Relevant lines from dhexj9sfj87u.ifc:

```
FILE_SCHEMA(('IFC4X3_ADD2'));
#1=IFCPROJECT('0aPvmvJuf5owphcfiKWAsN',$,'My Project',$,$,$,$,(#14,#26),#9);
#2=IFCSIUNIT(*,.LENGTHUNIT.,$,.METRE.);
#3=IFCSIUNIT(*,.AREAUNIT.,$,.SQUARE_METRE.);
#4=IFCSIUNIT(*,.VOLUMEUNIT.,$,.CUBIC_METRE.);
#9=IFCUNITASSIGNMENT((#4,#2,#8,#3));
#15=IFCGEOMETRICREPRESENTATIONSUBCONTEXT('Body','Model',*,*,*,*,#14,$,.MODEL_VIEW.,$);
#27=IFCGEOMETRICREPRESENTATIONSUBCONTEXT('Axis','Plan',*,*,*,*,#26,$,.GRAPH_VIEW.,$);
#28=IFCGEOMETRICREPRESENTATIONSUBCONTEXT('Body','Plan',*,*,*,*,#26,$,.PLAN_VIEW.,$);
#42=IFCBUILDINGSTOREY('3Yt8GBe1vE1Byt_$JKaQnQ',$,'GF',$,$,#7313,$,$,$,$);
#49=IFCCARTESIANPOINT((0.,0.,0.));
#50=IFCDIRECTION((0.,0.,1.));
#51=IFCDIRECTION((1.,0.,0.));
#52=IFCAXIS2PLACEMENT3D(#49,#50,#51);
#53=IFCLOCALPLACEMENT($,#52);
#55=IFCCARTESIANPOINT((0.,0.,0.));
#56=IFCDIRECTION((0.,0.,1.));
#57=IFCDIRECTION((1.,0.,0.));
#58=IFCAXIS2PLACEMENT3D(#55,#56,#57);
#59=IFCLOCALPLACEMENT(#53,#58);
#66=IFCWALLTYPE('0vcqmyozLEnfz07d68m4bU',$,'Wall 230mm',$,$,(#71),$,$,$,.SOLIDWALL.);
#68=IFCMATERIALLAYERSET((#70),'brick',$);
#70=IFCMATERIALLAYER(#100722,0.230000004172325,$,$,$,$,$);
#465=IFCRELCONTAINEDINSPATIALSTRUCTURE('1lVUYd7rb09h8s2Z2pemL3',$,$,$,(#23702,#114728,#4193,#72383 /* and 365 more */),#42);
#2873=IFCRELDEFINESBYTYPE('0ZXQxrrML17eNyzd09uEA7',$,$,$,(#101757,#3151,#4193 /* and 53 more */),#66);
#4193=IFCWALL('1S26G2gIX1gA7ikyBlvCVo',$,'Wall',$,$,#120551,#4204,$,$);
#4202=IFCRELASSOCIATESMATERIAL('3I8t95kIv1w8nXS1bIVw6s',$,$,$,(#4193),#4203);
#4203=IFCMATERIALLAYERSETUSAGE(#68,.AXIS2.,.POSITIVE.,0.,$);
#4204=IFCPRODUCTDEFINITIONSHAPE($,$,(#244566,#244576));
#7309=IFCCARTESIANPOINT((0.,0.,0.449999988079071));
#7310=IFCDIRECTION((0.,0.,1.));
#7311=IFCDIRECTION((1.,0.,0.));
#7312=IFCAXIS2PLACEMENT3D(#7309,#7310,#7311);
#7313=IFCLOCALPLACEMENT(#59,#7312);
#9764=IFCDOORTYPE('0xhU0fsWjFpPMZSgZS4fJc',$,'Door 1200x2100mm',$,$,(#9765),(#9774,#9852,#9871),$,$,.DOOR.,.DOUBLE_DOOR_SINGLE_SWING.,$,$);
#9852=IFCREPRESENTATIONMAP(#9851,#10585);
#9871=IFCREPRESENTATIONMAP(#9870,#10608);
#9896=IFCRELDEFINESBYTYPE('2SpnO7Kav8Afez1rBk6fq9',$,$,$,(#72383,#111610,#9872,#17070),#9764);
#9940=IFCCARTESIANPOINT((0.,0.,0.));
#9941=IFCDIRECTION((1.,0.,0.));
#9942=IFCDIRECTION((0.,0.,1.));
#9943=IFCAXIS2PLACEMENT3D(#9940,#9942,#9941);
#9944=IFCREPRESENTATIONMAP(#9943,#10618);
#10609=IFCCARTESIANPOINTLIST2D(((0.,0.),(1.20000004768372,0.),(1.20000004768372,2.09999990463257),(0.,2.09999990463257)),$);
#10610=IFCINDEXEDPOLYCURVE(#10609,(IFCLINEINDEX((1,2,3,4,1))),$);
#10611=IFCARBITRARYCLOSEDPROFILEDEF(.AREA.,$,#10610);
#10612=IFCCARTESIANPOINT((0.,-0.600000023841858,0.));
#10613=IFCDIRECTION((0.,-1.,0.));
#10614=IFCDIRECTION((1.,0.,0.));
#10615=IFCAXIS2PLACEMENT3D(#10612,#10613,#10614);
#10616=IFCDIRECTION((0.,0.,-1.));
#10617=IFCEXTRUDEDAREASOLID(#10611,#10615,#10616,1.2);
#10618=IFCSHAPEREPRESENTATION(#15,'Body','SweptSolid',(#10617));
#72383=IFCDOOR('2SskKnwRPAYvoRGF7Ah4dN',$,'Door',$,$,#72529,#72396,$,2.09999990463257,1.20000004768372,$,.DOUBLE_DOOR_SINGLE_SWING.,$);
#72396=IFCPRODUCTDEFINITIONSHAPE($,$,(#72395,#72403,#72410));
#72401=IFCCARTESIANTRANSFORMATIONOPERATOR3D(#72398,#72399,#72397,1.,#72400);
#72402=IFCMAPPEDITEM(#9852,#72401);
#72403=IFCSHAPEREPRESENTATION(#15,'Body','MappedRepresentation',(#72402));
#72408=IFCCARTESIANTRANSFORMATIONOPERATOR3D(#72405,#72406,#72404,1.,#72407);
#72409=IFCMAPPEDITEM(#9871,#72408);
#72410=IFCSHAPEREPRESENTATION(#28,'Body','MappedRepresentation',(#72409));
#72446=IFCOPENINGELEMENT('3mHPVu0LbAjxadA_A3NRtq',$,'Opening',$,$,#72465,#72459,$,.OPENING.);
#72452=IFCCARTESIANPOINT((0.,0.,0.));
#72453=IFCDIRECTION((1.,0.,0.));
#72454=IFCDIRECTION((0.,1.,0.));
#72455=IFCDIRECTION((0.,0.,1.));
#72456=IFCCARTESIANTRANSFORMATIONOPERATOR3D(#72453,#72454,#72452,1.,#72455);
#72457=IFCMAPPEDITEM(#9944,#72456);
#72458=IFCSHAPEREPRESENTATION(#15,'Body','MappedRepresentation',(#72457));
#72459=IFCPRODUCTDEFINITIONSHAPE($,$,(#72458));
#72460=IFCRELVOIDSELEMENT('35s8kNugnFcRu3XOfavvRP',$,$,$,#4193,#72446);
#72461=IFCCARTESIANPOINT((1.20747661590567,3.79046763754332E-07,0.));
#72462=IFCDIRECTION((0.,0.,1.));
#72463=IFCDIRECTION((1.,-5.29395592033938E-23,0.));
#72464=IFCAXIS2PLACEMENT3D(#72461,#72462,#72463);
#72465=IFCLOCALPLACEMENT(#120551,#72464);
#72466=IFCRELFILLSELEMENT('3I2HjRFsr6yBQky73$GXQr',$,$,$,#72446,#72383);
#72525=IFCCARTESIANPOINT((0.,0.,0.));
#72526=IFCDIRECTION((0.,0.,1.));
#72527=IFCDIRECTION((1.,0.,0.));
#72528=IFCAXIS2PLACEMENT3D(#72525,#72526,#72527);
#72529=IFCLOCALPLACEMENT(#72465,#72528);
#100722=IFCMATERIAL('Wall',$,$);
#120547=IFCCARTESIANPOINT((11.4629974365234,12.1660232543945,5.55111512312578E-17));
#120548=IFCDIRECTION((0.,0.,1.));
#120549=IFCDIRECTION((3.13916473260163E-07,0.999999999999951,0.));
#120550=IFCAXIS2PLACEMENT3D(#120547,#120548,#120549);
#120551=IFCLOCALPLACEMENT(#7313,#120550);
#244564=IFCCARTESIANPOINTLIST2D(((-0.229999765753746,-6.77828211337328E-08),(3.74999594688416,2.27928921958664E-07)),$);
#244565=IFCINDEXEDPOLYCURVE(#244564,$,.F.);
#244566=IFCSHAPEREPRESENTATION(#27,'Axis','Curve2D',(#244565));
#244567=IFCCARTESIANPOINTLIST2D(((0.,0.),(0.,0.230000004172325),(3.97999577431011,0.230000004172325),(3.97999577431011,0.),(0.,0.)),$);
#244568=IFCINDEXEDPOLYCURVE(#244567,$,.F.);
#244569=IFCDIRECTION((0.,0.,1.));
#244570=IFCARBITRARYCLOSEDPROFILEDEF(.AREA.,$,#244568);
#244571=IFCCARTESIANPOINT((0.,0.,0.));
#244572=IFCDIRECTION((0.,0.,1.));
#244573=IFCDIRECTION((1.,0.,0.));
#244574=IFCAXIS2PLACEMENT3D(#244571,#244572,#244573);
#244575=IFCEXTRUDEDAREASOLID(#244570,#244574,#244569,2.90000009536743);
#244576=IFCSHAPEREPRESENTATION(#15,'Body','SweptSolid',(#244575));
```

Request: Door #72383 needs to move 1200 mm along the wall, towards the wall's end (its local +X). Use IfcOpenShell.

```python
import ifcopenshell
import ifcopenshell.api.geometry
import ifcopenshell.util.placement

model = ifcopenshell.open("dhexj9sfj87u.ifc")

door = model.by_guid("2SskKnwRPAYvoRGF7Ah4dN")
opening = door.FillsVoids[0].RelatingOpeningElement
wall = opening.VoidsElements[0].RelatingBuildingElement

wall_matrix = ifcopenshell.util.placement.get_local_placement(wall.ObjectPlacement)
shift = wall_matrix[:3, 0] * 1.2
before = ifcopenshell.util.placement.get_local_placement(door.ObjectPlacement)[:3, 3].copy()

# The door is placed relative to its opening, so it follows when the opening moves.
matrix = ifcopenshell.util.placement.get_local_placement(opening.ObjectPlacement)
matrix[:3, 3] += shift
ifcopenshell.api.geometry.edit_object_placement(
    model, product=opening, matrix=matrix, is_si=False, should_transform_children=True
)

after = ifcopenshell.util.placement.get_local_placement(door.ObjectPlacement)[:3, 3]
print("door moved by", (after - before).round(3) + 0.0)

model.write("dhexj9sfj87u_v2.ifc")
```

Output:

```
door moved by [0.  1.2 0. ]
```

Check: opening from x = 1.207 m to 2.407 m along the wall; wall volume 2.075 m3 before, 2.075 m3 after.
